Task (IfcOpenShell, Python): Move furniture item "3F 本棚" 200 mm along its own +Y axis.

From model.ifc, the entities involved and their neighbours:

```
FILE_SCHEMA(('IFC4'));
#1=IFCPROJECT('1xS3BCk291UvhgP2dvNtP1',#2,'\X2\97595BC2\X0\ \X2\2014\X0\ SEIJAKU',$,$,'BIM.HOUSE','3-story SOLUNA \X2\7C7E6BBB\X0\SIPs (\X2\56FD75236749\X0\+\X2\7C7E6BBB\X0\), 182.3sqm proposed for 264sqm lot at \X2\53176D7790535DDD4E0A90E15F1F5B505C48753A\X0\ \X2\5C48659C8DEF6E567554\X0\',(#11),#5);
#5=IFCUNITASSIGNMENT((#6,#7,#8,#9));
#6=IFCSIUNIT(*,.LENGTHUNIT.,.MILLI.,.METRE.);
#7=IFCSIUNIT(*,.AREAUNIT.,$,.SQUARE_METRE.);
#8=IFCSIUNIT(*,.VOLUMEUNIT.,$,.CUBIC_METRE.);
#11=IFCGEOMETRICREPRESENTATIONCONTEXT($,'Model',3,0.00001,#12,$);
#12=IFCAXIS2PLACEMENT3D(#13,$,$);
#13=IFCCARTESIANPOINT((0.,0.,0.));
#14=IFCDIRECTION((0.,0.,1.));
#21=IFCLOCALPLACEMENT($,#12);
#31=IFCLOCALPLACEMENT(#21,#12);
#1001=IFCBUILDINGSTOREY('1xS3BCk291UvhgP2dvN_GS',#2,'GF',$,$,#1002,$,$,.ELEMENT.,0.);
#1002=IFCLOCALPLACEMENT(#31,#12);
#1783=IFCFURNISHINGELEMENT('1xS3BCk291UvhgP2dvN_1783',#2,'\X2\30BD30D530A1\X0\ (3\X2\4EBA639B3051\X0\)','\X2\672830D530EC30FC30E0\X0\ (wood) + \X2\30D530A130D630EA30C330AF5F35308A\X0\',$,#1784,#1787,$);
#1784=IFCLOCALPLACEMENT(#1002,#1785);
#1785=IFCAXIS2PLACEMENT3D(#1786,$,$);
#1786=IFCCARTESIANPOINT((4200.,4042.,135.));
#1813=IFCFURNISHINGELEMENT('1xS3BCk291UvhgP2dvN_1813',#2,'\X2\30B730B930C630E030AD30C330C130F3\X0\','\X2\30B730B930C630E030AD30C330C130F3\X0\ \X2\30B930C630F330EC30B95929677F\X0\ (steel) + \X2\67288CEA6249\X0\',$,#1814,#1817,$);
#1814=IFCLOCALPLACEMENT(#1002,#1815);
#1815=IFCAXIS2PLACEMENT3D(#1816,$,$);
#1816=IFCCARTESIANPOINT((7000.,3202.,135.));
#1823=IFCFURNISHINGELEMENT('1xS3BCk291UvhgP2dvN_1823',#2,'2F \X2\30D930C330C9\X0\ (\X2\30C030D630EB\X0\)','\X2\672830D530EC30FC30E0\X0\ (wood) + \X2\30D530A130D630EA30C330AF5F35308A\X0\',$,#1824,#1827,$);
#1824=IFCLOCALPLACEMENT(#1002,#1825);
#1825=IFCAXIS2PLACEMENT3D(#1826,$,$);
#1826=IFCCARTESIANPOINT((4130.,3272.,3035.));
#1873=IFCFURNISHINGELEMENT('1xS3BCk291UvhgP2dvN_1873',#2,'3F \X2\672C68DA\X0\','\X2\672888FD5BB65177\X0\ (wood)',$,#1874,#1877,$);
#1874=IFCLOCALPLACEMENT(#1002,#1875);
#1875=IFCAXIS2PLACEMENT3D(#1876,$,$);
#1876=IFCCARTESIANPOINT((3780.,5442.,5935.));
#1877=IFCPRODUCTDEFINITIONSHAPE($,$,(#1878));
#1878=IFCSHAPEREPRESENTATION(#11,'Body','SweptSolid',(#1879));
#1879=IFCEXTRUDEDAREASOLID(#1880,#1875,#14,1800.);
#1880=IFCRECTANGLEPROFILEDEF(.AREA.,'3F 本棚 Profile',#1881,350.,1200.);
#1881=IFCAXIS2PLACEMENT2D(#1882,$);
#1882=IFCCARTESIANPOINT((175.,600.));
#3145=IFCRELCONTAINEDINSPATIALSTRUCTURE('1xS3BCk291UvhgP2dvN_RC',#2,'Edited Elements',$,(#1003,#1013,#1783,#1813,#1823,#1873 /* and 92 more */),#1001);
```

```python
import ifcopenshell
import ifcopenshell.api.geometry
import ifcopenshell.util.placement

model = ifcopenshell.open("model.ifc")

item = model.by_guid("1xS3BCk291UvhgP2dvN_1873")
matrix = ifcopenshell.util.placement.get_local_placement(item.ObjectPlacement)
matrix[:3, 3] += matrix[:3, 1] * 200.0
ifcopenshell.api.geometry.edit_object_placement(model, product=item, matrix=matrix, is_si=False)

print(ifcopenshell.util.placement.get_local_placement(item.ObjectPlacement).round(3) + 0.0)

model.write("model_v2.ifc")
```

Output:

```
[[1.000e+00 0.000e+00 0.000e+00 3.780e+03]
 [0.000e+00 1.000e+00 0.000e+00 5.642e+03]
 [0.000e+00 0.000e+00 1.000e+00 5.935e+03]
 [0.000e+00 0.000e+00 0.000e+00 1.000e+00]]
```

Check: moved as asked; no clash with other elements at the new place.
